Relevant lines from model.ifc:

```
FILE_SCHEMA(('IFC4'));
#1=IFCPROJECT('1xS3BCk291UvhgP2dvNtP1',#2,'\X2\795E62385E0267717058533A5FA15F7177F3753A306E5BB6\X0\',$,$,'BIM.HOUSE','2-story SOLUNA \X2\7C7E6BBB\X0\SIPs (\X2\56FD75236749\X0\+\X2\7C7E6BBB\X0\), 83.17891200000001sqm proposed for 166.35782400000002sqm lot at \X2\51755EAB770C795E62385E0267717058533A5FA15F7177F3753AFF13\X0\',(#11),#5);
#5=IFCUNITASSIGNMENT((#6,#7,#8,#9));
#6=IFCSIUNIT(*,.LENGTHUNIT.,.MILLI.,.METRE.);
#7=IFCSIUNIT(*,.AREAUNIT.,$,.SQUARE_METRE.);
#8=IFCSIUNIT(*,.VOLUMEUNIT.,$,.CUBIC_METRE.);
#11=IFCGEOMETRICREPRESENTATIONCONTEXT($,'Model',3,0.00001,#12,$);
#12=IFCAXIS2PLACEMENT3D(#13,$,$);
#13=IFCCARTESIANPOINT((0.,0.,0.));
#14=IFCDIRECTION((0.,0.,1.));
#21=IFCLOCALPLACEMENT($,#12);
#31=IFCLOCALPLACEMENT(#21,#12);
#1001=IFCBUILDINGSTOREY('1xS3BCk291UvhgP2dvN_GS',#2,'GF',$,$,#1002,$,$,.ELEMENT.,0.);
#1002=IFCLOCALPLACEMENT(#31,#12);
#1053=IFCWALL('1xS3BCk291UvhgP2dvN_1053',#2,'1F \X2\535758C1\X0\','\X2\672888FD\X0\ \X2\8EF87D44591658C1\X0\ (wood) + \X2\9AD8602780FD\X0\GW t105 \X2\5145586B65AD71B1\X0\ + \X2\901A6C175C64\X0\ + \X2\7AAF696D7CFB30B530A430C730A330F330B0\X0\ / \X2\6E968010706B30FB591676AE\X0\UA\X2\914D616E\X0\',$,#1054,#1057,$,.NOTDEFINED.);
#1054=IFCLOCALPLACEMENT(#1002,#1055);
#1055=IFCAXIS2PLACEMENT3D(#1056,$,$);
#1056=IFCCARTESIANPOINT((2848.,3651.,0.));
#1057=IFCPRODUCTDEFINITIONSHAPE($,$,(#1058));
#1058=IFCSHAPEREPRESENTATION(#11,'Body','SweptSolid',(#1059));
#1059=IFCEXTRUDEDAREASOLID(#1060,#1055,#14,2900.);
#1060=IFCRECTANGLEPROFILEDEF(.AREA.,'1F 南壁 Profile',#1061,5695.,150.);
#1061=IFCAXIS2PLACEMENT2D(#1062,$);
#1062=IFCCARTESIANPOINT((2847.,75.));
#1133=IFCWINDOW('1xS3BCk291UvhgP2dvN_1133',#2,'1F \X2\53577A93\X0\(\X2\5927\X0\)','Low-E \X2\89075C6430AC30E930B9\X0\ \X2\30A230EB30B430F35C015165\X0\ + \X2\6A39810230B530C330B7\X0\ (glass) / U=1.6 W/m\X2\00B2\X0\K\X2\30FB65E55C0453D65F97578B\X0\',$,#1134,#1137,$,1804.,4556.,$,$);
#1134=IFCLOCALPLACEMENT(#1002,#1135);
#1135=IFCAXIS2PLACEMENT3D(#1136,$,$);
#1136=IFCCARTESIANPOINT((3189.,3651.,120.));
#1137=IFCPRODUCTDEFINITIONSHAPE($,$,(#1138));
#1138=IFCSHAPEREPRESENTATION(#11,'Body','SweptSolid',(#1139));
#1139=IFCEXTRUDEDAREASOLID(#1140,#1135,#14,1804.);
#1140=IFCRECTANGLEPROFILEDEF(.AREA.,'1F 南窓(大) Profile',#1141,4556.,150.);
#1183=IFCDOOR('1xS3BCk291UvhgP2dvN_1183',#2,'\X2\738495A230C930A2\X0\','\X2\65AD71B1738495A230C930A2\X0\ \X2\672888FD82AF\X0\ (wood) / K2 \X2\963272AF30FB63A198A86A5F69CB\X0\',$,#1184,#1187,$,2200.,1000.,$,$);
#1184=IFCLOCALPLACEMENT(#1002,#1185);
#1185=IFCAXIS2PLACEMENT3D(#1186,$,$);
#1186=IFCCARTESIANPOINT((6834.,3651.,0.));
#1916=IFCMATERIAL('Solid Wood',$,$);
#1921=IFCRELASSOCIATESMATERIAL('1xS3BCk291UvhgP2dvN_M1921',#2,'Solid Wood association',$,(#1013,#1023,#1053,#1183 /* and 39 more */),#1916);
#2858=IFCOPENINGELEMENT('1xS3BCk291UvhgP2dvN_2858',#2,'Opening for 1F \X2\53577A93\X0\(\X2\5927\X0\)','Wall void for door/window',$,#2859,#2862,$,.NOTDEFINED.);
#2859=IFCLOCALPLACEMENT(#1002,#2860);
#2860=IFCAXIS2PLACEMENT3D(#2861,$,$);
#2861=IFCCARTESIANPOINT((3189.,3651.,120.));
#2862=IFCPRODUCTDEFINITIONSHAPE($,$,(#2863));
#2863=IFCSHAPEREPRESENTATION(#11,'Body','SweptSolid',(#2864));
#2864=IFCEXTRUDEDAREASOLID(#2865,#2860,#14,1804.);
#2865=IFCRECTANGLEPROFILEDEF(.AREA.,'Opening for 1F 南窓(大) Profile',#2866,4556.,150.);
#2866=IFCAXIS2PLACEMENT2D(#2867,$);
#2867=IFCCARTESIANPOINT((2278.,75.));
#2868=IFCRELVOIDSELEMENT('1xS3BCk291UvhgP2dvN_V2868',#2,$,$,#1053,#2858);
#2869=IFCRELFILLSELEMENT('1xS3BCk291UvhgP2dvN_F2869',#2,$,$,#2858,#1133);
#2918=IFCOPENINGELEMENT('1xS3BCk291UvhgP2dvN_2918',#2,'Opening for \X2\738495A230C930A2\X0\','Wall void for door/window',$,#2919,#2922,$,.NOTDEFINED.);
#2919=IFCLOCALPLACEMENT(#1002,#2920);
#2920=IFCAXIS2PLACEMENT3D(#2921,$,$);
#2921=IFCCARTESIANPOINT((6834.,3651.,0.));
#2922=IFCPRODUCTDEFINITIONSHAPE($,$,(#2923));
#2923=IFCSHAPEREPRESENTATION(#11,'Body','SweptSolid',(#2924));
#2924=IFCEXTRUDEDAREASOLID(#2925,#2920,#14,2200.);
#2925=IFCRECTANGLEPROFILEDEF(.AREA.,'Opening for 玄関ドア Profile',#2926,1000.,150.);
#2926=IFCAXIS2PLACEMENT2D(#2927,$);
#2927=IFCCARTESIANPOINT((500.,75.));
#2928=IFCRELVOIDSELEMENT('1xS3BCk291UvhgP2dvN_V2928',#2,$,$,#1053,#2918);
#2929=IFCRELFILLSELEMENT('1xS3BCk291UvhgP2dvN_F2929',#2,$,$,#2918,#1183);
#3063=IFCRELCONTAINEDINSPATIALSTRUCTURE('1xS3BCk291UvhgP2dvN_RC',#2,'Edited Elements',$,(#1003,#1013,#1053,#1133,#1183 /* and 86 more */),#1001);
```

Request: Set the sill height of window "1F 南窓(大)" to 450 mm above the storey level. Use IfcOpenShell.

```python
import numpy as np
import ifcopenshell
import ifcopenshell.api.geometry
import ifcopenshell.geom
import ifcopenshell.util.element
import ifcopenshell.util.placement
import ifcopenshell.util.shape
import ifcopenshell.util.unit

model = ifcopenshell.open("model.ifc")
unit_scale = ifcopenshell.util.unit.calculate_unit_scale(model)

window = model.by_guid("1xS3BCk291UvhgP2dvN_1133")
opening = window.FillsVoids[0].RelatingOpeningElement
storey = ifcopenshell.util.element.get_container(window, ifc_class="IfcBuildingStorey")
level = ifcopenshell.util.placement.get_local_placement(storey.ObjectPlacement)[2, 3]

# The opening's origin need not be at the sill, so measure its lowest point.
shape = ifcopenshell.geom.create_shape(ifcopenshell.geom.settings(), opening)
bottom = ifcopenshell.util.shape.get_shape_bottom_elevation(shape, shape.geometry) / unit_scale
dz = level + 0.45 / unit_scale - bottom

shift = np.array([0.0, 0.0, dz])
# The window is not placed relative to its opening, so move both.
for product in (opening, window):
    matrix = ifcopenshell.util.placement.get_local_placement(product.ObjectPlacement)
    matrix[:3, 3] += shift
    ifcopenshell.api.geometry.edit_object_placement(model, product=product, matrix=matrix, is_si=False)

print(f"moved by {dz * unit_scale:+.3f} m")

model.write("model_updated.ifc")
```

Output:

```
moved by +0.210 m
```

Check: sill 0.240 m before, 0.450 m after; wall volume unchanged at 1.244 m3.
